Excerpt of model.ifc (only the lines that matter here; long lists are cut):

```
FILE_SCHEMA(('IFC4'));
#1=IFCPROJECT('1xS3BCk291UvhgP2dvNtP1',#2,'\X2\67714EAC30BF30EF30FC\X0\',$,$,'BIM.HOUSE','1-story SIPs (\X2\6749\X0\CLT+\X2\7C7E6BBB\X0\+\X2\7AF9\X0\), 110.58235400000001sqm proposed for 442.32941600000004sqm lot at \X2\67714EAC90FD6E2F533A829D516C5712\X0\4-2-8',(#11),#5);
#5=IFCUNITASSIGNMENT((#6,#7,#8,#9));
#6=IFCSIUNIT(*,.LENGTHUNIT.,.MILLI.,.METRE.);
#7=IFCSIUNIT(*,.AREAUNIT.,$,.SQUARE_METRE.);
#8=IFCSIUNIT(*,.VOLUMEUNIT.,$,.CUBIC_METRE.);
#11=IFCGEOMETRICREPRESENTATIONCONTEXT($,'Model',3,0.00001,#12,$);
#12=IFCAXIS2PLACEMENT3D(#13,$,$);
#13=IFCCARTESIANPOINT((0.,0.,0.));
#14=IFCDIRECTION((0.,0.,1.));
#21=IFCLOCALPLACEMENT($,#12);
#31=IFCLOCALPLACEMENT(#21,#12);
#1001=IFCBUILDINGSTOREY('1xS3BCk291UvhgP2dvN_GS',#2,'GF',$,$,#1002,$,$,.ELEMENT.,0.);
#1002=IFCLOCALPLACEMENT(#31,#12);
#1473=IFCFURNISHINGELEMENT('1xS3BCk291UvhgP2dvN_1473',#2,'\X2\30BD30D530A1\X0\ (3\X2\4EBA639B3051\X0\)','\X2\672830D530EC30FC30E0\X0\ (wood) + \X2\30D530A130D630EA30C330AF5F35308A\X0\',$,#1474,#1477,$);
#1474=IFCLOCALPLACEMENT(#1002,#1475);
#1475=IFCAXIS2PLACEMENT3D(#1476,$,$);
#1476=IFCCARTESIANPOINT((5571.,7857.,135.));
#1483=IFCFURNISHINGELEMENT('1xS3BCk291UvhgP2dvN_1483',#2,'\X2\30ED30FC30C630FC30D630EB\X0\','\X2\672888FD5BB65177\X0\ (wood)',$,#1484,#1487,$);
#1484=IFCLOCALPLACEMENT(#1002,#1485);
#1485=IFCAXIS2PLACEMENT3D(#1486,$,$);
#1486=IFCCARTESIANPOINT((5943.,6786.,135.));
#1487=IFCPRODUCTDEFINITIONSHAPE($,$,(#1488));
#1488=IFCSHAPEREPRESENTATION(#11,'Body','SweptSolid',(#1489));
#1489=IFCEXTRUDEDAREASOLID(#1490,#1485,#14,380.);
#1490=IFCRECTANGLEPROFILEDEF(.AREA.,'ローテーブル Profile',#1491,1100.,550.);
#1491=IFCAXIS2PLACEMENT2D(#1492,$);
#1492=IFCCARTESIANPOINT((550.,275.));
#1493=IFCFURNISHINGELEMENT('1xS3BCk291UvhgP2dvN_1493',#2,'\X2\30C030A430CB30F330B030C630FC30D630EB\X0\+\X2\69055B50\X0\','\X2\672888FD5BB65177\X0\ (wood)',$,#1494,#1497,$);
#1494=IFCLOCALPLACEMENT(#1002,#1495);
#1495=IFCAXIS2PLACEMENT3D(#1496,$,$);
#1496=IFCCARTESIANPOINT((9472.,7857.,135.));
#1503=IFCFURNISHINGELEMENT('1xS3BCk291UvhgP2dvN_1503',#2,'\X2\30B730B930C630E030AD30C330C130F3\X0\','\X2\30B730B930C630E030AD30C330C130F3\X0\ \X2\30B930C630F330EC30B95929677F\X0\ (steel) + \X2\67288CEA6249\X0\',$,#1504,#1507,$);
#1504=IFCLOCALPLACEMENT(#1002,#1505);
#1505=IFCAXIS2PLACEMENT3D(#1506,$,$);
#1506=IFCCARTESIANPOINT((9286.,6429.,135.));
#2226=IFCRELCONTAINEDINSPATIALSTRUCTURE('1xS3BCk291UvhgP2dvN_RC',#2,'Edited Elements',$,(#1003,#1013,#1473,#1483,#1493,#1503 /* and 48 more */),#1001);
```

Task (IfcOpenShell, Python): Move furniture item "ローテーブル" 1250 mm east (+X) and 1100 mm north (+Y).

```python
import ifcopenshell
import ifcopenshell.api.geometry
import ifcopenshell.util.placement

model = ifcopenshell.open("model.ifc")

item = model.by_guid("1xS3BCk291UvhgP2dvN_1483")
matrix = ifcopenshell.util.placement.get_local_placement(item.ObjectPlacement)
matrix[0, 3] += 1250.0
matrix[1, 3] += 1100.0
ifcopenshell.api.geometry.edit_object_placement(model, product=item, matrix=matrix, is_si=False)

print(ifcopenshell.util.placement.get_local_placement(item.ObjectPlacement).round(3) + 0.0)

model.write("model_v2.ifc")
```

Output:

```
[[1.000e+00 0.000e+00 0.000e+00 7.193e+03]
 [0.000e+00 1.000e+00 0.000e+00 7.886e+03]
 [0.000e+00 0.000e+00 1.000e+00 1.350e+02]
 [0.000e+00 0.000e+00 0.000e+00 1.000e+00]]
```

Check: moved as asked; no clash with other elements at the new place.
